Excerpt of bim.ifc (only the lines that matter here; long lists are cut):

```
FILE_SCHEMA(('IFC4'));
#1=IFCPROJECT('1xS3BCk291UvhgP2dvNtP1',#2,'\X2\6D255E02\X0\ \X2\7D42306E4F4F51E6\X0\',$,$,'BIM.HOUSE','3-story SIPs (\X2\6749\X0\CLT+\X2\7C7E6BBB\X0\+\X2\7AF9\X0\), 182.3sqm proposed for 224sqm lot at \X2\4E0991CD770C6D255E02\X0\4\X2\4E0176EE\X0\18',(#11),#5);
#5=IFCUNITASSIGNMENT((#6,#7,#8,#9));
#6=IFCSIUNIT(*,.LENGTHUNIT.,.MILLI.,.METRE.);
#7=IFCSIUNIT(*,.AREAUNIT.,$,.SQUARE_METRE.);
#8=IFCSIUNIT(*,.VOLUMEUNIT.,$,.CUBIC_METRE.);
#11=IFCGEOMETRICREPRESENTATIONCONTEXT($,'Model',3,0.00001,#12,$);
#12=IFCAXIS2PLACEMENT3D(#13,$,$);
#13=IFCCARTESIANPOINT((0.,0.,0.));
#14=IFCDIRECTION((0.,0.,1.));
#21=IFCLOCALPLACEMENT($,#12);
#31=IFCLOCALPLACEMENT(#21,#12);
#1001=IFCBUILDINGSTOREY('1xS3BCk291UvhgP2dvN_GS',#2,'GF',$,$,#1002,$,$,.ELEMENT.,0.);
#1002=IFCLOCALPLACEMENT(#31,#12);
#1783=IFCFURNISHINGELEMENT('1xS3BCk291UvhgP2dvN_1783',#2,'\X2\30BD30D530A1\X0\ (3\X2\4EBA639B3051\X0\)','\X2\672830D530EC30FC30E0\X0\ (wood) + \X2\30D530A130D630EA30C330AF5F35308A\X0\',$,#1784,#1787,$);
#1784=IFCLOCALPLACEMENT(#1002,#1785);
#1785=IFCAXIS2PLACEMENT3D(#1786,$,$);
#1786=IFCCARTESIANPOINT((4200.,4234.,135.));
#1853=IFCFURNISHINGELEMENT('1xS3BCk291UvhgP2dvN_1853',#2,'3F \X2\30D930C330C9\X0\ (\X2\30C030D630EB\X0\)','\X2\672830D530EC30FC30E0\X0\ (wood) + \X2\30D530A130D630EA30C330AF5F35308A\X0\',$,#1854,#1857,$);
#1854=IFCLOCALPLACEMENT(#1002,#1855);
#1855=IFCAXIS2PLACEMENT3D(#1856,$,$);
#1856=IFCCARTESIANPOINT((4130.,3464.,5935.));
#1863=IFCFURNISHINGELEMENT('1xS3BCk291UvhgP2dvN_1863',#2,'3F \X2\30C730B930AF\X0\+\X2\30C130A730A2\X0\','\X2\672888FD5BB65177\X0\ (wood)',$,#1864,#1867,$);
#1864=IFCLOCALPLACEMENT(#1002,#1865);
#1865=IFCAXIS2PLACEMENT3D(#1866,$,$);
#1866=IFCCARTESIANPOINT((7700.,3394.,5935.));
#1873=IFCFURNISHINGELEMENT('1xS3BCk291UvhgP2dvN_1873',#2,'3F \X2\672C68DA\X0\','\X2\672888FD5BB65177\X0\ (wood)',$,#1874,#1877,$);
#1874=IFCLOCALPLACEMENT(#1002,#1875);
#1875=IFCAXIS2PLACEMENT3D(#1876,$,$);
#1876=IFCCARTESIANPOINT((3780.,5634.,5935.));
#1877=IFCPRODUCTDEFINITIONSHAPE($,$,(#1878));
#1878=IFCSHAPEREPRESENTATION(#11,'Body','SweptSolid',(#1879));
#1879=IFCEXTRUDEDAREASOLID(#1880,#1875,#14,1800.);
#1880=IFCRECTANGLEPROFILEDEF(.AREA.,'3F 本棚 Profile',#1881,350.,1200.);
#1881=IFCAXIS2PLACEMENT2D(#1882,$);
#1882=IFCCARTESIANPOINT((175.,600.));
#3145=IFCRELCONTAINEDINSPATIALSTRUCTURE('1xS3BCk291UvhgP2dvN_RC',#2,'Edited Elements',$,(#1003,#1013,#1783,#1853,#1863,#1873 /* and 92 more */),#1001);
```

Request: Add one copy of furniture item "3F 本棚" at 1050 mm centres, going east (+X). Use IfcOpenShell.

```python
import numpy as np
import ifcopenshell
import ifcopenshell.api.geometry
import ifcopenshell.api.root
import ifcopenshell.util.element
import ifcopenshell.util.placement
import ifcopenshell.util.unit

model = ifcopenshell.open("bim.ifc")
unit_scale = ifcopenshell.util.unit.calculate_unit_scale(model)


def reuse_history(source, copy):
    """copy_class also copies each property set's owner history, people and application; keep the originals."""
    for rel in copy.IsDefinedBy:
        if rel.is_a("IfcRelDefinesByProperties") and (history := rel.RelatingPropertyDefinition.OwnerHistory):
            rel.RelatingPropertyDefinition.OwnerHistory = source.OwnerHistory
            ifcopenshell.util.element.remove_deep2(model, history)


source = model.by_guid("1xS3BCk291UvhgP2dvN_1873")
base = ifcopenshell.util.placement.get_local_placement(source.ObjectPlacement)
step = np.array([1.0, 0.0, 0.0]) * 1.05 / unit_scale

for i in range(1, 2):
    copy = ifcopenshell.api.root.copy_class(model, product=source)
    copy.Representation = ifcopenshell.util.element.copy_deep(
        model, source.Representation, exclude=["IfcGeometricRepresentationContext", "IfcRepresentationMap"]
    )
    reuse_history(source, copy)
    matrix = base.copy()
    matrix[:3, 3] += i * step
    print("added at", matrix[:3, 3].round(3) + 0.0)
    ifcopenshell.api.geometry.edit_object_placement(model, product=copy, matrix=matrix, is_si=False)

model.write("bim_edited.ifc")
```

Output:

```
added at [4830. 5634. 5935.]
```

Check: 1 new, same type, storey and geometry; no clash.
